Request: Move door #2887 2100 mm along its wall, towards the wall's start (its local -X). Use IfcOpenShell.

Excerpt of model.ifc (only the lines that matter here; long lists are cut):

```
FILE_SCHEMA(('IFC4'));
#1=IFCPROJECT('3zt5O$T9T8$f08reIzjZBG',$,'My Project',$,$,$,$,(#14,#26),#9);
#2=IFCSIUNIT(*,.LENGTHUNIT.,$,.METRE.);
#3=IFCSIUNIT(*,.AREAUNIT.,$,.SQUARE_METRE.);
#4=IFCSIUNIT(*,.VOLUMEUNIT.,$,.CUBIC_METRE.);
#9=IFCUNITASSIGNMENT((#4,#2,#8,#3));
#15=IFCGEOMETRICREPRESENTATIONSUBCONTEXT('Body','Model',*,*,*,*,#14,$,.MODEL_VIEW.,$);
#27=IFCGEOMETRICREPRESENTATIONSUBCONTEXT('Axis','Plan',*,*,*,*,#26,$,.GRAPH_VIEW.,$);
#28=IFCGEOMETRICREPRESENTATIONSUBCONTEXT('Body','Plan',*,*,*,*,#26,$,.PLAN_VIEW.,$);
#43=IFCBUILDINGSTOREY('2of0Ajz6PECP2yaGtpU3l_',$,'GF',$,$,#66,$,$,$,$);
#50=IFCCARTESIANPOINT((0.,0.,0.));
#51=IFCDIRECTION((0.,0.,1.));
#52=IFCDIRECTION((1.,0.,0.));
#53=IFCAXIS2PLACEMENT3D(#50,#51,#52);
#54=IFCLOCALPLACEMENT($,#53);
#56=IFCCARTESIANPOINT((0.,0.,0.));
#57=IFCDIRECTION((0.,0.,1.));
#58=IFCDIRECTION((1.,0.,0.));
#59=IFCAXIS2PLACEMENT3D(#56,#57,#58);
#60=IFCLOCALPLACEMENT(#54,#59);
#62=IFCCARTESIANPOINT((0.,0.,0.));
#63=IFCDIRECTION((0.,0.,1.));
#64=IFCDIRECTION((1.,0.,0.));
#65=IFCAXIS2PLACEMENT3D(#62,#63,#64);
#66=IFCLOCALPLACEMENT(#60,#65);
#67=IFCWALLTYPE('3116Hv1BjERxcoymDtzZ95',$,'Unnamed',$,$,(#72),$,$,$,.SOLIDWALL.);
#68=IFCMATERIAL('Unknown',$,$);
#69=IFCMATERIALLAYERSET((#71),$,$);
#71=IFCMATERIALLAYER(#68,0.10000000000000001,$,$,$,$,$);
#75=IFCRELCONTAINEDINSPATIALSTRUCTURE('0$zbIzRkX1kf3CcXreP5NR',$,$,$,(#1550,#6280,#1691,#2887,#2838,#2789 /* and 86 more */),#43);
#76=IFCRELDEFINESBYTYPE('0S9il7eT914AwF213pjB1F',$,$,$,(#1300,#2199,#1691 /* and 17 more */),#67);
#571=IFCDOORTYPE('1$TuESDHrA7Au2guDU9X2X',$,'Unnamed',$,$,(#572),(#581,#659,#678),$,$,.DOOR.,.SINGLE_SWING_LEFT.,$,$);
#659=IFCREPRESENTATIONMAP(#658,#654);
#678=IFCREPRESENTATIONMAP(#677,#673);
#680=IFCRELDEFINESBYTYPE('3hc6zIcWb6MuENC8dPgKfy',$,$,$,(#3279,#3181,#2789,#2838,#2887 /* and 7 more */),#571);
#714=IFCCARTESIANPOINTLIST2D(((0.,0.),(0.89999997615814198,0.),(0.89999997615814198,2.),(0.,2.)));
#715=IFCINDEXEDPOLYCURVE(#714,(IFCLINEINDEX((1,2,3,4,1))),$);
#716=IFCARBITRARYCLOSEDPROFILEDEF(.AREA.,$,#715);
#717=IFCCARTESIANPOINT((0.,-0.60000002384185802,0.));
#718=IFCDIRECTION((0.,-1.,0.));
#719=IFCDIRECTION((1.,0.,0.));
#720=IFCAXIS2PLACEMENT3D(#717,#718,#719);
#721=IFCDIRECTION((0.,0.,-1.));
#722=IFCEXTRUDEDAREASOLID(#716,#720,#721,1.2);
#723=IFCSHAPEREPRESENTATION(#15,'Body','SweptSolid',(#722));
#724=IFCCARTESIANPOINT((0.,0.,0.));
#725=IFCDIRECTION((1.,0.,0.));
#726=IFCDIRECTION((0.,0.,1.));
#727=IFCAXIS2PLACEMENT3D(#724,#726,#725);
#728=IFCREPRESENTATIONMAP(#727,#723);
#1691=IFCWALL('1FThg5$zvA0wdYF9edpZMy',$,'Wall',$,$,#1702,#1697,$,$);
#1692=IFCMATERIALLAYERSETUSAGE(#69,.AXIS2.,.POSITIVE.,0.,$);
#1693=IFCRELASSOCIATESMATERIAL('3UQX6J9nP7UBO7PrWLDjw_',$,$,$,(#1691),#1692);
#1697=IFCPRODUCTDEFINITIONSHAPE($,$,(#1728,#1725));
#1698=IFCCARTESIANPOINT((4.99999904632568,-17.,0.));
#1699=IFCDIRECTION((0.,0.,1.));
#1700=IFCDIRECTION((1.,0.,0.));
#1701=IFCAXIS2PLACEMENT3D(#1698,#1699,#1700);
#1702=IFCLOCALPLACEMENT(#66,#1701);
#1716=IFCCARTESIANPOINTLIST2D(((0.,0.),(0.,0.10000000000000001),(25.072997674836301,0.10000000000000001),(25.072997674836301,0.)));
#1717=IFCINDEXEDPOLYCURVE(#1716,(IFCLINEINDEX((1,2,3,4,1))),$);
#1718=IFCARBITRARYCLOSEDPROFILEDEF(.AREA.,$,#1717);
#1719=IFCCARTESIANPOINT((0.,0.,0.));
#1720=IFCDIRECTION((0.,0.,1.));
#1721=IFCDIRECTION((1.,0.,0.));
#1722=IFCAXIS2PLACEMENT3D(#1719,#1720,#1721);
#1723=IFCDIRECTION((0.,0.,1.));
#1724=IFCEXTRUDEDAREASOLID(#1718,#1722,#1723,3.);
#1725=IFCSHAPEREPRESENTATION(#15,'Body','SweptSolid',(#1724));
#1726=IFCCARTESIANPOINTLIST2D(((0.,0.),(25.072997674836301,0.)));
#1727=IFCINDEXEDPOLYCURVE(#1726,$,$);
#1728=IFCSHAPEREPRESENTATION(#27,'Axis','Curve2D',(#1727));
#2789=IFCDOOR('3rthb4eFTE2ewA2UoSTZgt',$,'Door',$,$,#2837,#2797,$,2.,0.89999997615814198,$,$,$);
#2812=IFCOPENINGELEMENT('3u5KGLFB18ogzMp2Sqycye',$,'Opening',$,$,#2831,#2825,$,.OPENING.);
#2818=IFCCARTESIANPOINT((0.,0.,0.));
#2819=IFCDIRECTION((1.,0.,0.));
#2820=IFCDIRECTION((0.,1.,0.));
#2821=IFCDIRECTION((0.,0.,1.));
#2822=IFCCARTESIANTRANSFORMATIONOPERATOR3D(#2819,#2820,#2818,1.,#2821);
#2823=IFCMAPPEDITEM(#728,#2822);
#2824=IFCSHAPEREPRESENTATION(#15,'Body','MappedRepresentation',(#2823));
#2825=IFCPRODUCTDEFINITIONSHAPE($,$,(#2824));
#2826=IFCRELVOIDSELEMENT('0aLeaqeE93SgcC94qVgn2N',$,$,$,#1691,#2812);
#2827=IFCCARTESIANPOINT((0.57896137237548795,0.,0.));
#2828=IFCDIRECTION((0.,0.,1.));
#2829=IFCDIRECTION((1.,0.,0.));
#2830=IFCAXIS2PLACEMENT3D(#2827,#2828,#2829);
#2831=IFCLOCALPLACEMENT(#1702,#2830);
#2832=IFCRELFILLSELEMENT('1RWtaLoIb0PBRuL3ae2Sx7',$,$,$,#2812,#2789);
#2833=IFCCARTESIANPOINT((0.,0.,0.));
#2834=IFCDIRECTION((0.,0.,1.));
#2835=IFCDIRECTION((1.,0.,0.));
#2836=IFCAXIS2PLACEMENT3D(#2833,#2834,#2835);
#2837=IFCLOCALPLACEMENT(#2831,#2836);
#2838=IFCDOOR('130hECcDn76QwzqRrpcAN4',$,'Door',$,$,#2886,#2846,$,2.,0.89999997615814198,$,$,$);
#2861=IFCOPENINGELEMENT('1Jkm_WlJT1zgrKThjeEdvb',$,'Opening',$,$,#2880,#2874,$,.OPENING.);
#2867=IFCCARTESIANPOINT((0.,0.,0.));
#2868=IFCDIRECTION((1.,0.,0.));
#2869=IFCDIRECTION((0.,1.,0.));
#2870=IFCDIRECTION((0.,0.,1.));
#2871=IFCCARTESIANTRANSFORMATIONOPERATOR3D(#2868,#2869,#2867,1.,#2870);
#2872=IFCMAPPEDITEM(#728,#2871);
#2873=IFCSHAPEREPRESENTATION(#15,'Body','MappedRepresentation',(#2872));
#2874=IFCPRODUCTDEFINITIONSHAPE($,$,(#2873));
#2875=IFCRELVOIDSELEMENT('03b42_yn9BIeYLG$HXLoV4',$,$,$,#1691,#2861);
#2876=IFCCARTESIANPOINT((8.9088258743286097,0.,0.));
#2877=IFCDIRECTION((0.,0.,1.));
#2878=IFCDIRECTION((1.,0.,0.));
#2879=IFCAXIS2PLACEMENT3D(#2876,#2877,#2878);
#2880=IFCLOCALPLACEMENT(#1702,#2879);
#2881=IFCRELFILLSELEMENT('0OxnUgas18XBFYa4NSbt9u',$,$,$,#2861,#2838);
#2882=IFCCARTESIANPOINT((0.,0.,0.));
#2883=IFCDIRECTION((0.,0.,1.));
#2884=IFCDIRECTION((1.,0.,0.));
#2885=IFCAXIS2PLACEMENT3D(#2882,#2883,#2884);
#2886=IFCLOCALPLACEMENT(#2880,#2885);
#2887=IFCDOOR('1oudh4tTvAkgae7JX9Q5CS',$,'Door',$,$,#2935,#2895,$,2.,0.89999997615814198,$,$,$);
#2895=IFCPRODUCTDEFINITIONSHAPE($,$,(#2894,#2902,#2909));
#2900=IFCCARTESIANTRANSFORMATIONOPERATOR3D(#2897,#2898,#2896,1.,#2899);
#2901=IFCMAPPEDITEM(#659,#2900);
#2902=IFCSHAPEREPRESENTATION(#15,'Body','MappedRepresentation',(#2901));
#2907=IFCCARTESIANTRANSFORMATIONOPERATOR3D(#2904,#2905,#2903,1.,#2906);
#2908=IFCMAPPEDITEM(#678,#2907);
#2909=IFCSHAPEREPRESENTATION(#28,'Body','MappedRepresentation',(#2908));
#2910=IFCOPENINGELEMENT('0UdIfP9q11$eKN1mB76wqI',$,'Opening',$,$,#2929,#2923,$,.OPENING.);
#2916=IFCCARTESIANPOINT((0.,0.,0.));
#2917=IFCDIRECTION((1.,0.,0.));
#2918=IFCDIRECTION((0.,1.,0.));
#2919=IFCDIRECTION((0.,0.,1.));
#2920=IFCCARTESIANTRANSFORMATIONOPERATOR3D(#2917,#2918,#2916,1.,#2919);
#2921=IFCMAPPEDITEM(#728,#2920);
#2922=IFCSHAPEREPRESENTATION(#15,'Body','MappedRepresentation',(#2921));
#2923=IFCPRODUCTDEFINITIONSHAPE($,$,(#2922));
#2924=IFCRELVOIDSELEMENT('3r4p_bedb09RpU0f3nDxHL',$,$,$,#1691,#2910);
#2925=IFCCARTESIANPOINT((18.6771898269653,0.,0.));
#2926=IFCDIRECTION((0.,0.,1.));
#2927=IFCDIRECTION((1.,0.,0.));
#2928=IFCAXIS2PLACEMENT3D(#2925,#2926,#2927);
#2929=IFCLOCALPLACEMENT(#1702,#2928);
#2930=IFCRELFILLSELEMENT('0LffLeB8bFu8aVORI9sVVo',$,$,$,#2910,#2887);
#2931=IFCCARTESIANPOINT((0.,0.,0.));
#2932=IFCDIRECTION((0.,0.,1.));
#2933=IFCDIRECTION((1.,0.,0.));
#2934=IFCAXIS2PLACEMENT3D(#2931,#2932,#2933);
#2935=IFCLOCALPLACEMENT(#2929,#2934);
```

```python
import ifcopenshell
import ifcopenshell.api.geometry
import ifcopenshell.util.placement

model = ifcopenshell.open("model.ifc")

door = model.by_guid("1oudh4tTvAkgae7JX9Q5CS")
opening = door.FillsVoids[0].RelatingOpeningElement
wall = opening.VoidsElements[0].RelatingBuildingElement

wall_matrix = ifcopenshell.util.placement.get_local_placement(wall.ObjectPlacement)
shift = wall_matrix[:3, 0] * -2.1
before = ifcopenshell.util.placement.get_local_placement(door.ObjectPlacement)[:3, 3].copy()

# The door is placed relative to its opening, so it follows when the opening moves.
matrix = ifcopenshell.util.placement.get_local_placement(opening.ObjectPlacement)
matrix[:3, 3] += shift
ifcopenshell.api.geometry.edit_object_placement(
    model, product=opening, matrix=matrix, is_si=False, should_transform_children=True
)

after = ifcopenshell.util.placement.get_local_placement(door.ObjectPlacement)[:3, 3]
print("door moved by", (after - before).round(3) + 0.0)

model.write("model_rev.ifc")
```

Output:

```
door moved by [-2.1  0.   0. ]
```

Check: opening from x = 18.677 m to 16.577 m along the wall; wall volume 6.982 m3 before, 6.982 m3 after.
